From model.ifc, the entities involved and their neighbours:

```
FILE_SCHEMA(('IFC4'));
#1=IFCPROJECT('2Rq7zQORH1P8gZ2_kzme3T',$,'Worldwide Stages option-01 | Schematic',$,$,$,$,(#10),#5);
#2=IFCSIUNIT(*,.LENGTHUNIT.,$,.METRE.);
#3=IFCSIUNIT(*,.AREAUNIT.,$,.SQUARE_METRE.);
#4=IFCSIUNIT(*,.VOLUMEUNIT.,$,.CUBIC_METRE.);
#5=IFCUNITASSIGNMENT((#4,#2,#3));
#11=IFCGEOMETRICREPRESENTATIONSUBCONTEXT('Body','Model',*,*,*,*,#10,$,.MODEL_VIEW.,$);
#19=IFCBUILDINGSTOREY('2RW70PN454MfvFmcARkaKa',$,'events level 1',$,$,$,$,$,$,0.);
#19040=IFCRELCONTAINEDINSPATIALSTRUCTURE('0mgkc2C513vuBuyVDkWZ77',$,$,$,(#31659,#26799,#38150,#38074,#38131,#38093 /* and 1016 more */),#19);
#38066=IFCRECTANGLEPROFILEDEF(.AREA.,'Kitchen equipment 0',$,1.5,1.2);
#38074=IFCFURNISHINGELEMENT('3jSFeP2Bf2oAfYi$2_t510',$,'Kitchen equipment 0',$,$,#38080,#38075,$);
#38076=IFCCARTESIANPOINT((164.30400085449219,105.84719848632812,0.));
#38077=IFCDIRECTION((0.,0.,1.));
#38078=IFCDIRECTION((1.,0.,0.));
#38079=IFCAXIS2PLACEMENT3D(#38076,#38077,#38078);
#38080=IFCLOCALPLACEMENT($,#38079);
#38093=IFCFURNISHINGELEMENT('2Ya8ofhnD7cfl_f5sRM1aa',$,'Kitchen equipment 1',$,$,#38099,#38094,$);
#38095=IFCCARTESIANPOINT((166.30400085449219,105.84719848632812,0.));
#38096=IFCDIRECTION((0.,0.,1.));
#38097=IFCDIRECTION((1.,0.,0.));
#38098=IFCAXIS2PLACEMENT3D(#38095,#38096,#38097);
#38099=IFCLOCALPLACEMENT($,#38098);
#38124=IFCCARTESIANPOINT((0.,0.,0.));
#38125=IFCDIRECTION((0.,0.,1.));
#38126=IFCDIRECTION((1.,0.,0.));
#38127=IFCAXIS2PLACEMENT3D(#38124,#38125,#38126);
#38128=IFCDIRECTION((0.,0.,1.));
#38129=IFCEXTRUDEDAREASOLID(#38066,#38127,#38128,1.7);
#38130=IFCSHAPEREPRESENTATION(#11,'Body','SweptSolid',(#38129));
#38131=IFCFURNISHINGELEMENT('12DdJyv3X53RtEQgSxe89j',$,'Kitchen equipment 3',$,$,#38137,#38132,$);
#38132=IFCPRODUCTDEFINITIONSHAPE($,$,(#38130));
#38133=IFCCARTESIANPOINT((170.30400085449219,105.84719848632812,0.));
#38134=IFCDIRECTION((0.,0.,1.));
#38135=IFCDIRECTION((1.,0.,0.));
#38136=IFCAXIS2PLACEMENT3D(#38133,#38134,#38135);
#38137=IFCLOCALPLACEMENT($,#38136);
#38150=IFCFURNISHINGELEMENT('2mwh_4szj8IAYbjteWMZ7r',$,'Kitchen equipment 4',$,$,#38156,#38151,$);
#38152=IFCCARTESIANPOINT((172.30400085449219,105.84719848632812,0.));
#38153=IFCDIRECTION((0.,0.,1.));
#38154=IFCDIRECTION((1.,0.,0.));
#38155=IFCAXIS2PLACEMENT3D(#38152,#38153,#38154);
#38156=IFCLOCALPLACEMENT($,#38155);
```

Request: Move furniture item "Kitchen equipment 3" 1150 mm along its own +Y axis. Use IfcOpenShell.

```python
import ifcopenshell
import ifcopenshell.api.geometry
import ifcopenshell.util.placement

model = ifcopenshell.open("model.ifc")

item = model.by_id(38131)
matrix = ifcopenshell.util.placement.get_local_placement(item.ObjectPlacement)
matrix[:3, 3] += matrix[:3, 1] * 1.15
ifcopenshell.api.geometry.edit_object_placement(model, product=item, matrix=matrix, is_si=False)

print(ifcopenshell.util.placement.get_local_placement(item.ObjectPlacement).round(3) + 0.0)

model.write("model_rev.ifc")
```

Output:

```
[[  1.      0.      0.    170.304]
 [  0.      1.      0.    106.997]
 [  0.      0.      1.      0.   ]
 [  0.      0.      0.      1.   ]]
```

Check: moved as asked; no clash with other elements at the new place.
